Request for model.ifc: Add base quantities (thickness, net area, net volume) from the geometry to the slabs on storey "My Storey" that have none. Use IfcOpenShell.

First a look at what the model holds.

```python
import ifcopenshell
import ifcopenshell.util.element
import ifcopenshell.util.unit

model = ifcopenshell.open("model.ifc")
print(model.schema)
for unit_type in ("LENGTHUNIT", "AREAUNIT", "VOLUMEUNIT"):
    print(unit_type, ifcopenshell.util.unit.calculate_unit_scale(model, unit_type))
storey = next(s for s in model.by_type("IfcBuildingStorey") if s.Name == "My Storey")
slabs = [e for e in ifcopenshell.util.element.get_decomposition(storey) if e.is_a("IfcSlab")]
for e in sorted(slabs, key=lambda e: e.id()):
    print(e.id(), e.is_a(), e.Name, list(ifcopenshell.util.element.get_psets(e, qtos_only=True)), sep=" | ")
```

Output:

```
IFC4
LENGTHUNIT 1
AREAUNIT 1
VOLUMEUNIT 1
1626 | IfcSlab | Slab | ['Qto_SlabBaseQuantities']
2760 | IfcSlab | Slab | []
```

```python
import ifcopenshell
import ifcopenshell.api.pset
import ifcopenshell.geom
import ifcopenshell.util.element
import ifcopenshell.util.shape
import ifcopenshell.util.unit

model = ifcopenshell.open("model.ifc")
unit_scale = ifcopenshell.util.unit.calculate_unit_scale(model)
area_scale = ifcopenshell.util.unit.calculate_unit_scale(model, "AREAUNIT")
volume_scale = ifcopenshell.util.unit.calculate_unit_scale(model, "VOLUMEUNIT")
settings = ifcopenshell.geom.settings()

storey = next(s for s in model.by_type("IfcBuildingStorey") if s.Name == "My Storey")
slabs = [e for e in ifcopenshell.util.element.get_decomposition(storey) if e.is_a("IfcSlab")]

for e in sorted(slabs, key=lambda e: e.id()):
    if ifcopenshell.util.element.get_psets(e, qtos_only=True, should_inherit=False):
        continue
    # Geometry comes back in metres, in the element's own axes.
    shape = ifcopenshell.geom.create_shape(settings, e)
    values = {
        "Width": ifcopenshell.util.shape.get_z(shape.geometry) / unit_scale,
        "NetArea": ifcopenshell.util.shape.get_footprint_area(shape.geometry) / area_scale,
        "NetVolume": ifcopenshell.util.shape.get_volume(shape.geometry) / volume_scale,
    }
    qto = ifcopenshell.api.pset.add_qto(model, product=e, name="Qto_SlabBaseQuantities")
    ifcopenshell.api.pset.edit_qto(model, qto=qto, properties=values)
    print(e.id(), {k: round(v, 3) for k, v in values.items()})

model.write("model-out.ifc")
```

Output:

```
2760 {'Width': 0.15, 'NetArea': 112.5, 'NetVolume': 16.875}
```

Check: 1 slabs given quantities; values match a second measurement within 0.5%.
